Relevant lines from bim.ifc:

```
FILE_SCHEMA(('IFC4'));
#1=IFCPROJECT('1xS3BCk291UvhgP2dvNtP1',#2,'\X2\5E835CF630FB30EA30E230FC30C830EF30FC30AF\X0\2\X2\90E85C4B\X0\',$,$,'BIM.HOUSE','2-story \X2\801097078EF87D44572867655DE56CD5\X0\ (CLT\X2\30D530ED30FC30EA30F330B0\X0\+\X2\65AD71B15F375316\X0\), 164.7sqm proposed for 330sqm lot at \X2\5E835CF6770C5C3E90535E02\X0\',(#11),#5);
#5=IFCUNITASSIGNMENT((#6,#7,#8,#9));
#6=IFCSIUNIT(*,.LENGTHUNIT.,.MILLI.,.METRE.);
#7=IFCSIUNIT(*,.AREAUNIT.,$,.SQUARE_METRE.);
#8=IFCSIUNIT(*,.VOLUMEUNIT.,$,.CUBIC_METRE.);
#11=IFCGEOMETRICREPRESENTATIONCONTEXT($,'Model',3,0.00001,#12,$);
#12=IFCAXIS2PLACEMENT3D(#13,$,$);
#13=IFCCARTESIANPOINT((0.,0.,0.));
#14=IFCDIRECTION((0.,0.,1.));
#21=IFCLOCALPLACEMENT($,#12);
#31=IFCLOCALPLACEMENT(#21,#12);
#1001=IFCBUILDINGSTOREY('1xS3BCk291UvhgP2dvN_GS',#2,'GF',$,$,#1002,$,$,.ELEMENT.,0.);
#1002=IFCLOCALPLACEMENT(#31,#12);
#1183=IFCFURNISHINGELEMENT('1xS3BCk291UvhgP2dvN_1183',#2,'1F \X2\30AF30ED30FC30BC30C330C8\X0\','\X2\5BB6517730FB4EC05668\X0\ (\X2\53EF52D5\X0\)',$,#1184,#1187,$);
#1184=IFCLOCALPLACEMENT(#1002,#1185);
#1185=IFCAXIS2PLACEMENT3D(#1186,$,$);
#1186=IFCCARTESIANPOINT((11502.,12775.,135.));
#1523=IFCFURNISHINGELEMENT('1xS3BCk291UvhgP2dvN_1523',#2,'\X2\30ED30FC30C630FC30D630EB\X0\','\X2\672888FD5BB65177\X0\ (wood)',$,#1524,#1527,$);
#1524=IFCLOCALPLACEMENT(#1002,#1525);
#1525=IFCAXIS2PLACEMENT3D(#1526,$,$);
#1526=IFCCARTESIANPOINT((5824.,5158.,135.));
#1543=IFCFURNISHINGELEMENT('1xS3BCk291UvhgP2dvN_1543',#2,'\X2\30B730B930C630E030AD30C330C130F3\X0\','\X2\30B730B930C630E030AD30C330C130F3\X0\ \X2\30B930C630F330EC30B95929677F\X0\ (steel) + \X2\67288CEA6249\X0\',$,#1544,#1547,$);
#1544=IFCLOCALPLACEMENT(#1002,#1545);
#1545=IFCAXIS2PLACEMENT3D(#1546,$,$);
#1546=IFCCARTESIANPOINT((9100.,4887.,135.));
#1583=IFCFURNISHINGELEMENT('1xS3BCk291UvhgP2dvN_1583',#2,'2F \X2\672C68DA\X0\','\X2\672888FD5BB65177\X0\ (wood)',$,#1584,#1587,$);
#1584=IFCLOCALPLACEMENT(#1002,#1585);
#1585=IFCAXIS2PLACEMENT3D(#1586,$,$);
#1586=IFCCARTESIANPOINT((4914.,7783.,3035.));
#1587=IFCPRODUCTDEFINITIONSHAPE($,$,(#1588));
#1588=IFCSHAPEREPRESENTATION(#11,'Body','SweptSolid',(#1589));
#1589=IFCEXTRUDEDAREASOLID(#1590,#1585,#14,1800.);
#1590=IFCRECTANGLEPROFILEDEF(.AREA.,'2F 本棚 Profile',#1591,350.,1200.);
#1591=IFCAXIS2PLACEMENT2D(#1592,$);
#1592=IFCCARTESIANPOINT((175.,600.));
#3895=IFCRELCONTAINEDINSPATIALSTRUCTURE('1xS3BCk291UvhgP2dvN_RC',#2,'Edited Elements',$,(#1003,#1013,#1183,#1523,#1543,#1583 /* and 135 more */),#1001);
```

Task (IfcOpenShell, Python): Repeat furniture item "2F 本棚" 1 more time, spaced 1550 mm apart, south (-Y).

```python
import numpy as np
import ifcopenshell
import ifcopenshell.api.geometry
import ifcopenshell.api.root
import ifcopenshell.util.element
import ifcopenshell.util.placement
import ifcopenshell.util.unit

model = ifcopenshell.open("bim.ifc")
unit_scale = ifcopenshell.util.unit.calculate_unit_scale(model)


def reuse_history(source, copy):
    """copy_class also copies each property set's owner history, people and application; keep the originals."""
    for rel in copy.IsDefinedBy:
        if rel.is_a("IfcRelDefinesByProperties") and (history := rel.RelatingPropertyDefinition.OwnerHistory):
            rel.RelatingPropertyDefinition.OwnerHistory = source.OwnerHistory
            ifcopenshell.util.element.remove_deep2(model, history)


source = model.by_id(1583)
base = ifcopenshell.util.placement.get_local_placement(source.ObjectPlacement)
step = np.array([0.0, -1.0, 0.0]) * 1.55 / unit_scale

for i in range(1, 2):
    copy = ifcopenshell.api.root.copy_class(model, product=source)
    copy.Representation = ifcopenshell.util.element.copy_deep(
        model, source.Representation, exclude=["IfcGeometricRepresentationContext", "IfcRepresentationMap"]
    )
    reuse_history(source, copy)
    matrix = base.copy()
    matrix[:3, 3] += i * step
    print("added at", matrix[:3, 3].round(3) + 0.0)
    ifcopenshell.api.geometry.edit_object_placement(model, product=copy, matrix=matrix, is_si=False)

model.write("bim_updated.ifc")
```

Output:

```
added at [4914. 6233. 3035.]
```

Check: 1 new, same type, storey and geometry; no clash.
